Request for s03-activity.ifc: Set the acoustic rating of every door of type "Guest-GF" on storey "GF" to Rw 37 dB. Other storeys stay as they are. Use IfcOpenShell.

First a look at what the model holds.

```python
import ifcopenshell
import ifcopenshell.util.element

model = ifcopenshell.open("s03-activity.ifc")
print(model.schema)
storey = next(s for s in model.by_type("IfcBuildingStorey") if s.Name == "GF")
doors = [e for e in ifcopenshell.util.element.get_decomposition(storey) if e.is_a("IfcDoor")]
seen = {}
for e in doors:
    element_type = ifcopenshell.util.element.get_type(e)
    key = (element_type.Name if element_type != e and element_type else None, ifcopenshell.util.element.get_pset(e, "Pset_DoorCommon", "AcousticRating"))
    seen[key] = seen.get(key, 0) + 1
for (name, value), count in sorted(seen.items(), key=str):
    print(count, "x", name, "|", value)
```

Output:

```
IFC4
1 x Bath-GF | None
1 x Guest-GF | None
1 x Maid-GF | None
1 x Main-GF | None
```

```python
import ifcopenshell
import ifcopenshell.api.pset
import ifcopenshell.util.element

model = ifcopenshell.open("s03-activity.ifc")

storey = next(s for s in model.by_type("IfcBuildingStorey") if s.Name == "GF")
doors = [e for e in ifcopenshell.util.element.get_decomposition(storey) if e.is_a("IfcDoor")]

count = 0
for e in doors:
    element_type = ifcopenshell.util.element.get_type(e)
    if element_type in (None, e) or element_type.Name != "Guest-GF":
        continue
    # add_pset returns the element's existing set when there is one.
    pset = ifcopenshell.api.pset.add_pset(model, product=e, name="Pset_DoorCommon")
    ifcopenshell.api.pset.edit_pset(model, pset=pset, properties={"AcousticRating": "Rw 37 dB"})
    count += 1

print(count, "doors updated")

model.write("s03-activity_updated.ifc")
```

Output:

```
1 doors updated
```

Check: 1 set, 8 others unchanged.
